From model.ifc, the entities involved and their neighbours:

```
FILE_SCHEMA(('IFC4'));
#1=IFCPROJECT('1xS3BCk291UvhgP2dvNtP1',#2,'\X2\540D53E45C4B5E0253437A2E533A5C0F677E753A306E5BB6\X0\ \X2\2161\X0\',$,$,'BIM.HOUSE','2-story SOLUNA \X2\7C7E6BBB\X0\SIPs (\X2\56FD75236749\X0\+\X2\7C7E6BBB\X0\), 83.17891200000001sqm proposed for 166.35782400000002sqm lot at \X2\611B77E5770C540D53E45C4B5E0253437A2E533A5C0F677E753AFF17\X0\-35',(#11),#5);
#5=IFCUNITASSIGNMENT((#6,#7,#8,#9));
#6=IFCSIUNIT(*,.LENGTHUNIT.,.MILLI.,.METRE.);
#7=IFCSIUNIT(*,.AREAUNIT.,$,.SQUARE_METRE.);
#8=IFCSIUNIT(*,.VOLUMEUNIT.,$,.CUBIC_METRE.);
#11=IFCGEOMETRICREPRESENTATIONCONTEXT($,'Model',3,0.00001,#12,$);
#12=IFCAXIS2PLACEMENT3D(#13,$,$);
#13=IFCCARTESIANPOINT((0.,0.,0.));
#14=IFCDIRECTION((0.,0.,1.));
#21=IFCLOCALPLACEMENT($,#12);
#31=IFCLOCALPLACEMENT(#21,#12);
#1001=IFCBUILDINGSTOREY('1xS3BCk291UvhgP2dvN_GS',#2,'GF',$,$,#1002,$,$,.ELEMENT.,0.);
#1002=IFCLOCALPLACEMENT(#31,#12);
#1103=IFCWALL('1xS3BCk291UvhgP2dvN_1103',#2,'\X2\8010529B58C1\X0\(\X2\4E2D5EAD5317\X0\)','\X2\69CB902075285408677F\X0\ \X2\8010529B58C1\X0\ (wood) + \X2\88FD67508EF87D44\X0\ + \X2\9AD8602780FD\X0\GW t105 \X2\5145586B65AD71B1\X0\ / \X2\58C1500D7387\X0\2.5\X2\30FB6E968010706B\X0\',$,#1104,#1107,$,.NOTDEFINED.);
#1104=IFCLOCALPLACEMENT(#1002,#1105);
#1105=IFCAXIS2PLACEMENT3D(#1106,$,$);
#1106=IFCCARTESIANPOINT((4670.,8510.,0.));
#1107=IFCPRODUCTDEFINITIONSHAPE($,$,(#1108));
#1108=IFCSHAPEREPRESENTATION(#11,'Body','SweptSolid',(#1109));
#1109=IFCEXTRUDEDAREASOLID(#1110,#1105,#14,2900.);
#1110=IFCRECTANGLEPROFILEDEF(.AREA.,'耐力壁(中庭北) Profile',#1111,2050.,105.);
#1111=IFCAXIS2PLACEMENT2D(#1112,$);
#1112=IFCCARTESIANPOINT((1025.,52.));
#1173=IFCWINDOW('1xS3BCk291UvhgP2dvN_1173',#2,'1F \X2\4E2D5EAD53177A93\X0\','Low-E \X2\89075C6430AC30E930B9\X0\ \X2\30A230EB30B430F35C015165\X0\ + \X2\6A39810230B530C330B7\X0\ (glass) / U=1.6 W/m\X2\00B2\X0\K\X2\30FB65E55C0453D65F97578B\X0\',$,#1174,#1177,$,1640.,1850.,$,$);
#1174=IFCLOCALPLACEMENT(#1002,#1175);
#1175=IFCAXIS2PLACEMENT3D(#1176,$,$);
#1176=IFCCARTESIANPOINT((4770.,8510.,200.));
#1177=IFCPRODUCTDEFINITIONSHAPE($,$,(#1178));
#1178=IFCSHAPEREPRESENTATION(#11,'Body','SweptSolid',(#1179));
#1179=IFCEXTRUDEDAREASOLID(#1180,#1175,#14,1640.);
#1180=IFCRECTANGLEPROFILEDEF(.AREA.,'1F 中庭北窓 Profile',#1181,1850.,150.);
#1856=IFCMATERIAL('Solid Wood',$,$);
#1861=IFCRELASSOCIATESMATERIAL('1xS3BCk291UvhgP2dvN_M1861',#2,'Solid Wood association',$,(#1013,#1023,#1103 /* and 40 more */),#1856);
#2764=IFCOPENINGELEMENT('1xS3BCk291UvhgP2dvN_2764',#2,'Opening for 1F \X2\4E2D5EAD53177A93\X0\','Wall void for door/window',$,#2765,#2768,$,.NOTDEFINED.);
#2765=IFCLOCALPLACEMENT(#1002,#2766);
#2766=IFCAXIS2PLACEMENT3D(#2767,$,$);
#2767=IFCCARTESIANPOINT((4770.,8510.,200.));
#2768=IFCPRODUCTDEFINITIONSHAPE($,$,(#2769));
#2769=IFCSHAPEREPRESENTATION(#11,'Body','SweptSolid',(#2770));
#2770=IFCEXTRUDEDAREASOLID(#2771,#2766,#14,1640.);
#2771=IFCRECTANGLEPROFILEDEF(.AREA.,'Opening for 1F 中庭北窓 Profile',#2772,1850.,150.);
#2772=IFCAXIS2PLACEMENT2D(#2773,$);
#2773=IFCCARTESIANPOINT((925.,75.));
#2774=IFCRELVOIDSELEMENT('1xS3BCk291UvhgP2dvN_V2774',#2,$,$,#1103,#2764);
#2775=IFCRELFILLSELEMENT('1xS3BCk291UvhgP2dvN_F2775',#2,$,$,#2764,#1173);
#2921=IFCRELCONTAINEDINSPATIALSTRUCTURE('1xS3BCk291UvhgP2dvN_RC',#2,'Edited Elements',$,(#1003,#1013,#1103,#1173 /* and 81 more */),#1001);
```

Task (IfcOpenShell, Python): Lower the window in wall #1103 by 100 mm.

```python
import numpy as np
import ifcopenshell
import ifcopenshell.api.geometry
import ifcopenshell.util.placement
import ifcopenshell.util.unit

model = ifcopenshell.open("model.ifc")
unit_scale = ifcopenshell.util.unit.calculate_unit_scale(model)

window = model.by_id(1173)
opening = window.FillsVoids[0].RelatingOpeningElement
dz = -100.0

shift = np.array([0.0, 0.0, dz])
# The window is not placed relative to its opening, so move both.
for product in (opening, window):
    matrix = ifcopenshell.util.placement.get_local_placement(product.ObjectPlacement)
    matrix[:3, 3] += shift
    ifcopenshell.api.geometry.edit_object_placement(model, product=product, matrix=matrix, is_si=False)

print(f"moved by {dz * unit_scale:+.3f} m")

model.write("model-out.ifc")
```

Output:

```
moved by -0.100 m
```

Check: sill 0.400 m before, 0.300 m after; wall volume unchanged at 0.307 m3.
